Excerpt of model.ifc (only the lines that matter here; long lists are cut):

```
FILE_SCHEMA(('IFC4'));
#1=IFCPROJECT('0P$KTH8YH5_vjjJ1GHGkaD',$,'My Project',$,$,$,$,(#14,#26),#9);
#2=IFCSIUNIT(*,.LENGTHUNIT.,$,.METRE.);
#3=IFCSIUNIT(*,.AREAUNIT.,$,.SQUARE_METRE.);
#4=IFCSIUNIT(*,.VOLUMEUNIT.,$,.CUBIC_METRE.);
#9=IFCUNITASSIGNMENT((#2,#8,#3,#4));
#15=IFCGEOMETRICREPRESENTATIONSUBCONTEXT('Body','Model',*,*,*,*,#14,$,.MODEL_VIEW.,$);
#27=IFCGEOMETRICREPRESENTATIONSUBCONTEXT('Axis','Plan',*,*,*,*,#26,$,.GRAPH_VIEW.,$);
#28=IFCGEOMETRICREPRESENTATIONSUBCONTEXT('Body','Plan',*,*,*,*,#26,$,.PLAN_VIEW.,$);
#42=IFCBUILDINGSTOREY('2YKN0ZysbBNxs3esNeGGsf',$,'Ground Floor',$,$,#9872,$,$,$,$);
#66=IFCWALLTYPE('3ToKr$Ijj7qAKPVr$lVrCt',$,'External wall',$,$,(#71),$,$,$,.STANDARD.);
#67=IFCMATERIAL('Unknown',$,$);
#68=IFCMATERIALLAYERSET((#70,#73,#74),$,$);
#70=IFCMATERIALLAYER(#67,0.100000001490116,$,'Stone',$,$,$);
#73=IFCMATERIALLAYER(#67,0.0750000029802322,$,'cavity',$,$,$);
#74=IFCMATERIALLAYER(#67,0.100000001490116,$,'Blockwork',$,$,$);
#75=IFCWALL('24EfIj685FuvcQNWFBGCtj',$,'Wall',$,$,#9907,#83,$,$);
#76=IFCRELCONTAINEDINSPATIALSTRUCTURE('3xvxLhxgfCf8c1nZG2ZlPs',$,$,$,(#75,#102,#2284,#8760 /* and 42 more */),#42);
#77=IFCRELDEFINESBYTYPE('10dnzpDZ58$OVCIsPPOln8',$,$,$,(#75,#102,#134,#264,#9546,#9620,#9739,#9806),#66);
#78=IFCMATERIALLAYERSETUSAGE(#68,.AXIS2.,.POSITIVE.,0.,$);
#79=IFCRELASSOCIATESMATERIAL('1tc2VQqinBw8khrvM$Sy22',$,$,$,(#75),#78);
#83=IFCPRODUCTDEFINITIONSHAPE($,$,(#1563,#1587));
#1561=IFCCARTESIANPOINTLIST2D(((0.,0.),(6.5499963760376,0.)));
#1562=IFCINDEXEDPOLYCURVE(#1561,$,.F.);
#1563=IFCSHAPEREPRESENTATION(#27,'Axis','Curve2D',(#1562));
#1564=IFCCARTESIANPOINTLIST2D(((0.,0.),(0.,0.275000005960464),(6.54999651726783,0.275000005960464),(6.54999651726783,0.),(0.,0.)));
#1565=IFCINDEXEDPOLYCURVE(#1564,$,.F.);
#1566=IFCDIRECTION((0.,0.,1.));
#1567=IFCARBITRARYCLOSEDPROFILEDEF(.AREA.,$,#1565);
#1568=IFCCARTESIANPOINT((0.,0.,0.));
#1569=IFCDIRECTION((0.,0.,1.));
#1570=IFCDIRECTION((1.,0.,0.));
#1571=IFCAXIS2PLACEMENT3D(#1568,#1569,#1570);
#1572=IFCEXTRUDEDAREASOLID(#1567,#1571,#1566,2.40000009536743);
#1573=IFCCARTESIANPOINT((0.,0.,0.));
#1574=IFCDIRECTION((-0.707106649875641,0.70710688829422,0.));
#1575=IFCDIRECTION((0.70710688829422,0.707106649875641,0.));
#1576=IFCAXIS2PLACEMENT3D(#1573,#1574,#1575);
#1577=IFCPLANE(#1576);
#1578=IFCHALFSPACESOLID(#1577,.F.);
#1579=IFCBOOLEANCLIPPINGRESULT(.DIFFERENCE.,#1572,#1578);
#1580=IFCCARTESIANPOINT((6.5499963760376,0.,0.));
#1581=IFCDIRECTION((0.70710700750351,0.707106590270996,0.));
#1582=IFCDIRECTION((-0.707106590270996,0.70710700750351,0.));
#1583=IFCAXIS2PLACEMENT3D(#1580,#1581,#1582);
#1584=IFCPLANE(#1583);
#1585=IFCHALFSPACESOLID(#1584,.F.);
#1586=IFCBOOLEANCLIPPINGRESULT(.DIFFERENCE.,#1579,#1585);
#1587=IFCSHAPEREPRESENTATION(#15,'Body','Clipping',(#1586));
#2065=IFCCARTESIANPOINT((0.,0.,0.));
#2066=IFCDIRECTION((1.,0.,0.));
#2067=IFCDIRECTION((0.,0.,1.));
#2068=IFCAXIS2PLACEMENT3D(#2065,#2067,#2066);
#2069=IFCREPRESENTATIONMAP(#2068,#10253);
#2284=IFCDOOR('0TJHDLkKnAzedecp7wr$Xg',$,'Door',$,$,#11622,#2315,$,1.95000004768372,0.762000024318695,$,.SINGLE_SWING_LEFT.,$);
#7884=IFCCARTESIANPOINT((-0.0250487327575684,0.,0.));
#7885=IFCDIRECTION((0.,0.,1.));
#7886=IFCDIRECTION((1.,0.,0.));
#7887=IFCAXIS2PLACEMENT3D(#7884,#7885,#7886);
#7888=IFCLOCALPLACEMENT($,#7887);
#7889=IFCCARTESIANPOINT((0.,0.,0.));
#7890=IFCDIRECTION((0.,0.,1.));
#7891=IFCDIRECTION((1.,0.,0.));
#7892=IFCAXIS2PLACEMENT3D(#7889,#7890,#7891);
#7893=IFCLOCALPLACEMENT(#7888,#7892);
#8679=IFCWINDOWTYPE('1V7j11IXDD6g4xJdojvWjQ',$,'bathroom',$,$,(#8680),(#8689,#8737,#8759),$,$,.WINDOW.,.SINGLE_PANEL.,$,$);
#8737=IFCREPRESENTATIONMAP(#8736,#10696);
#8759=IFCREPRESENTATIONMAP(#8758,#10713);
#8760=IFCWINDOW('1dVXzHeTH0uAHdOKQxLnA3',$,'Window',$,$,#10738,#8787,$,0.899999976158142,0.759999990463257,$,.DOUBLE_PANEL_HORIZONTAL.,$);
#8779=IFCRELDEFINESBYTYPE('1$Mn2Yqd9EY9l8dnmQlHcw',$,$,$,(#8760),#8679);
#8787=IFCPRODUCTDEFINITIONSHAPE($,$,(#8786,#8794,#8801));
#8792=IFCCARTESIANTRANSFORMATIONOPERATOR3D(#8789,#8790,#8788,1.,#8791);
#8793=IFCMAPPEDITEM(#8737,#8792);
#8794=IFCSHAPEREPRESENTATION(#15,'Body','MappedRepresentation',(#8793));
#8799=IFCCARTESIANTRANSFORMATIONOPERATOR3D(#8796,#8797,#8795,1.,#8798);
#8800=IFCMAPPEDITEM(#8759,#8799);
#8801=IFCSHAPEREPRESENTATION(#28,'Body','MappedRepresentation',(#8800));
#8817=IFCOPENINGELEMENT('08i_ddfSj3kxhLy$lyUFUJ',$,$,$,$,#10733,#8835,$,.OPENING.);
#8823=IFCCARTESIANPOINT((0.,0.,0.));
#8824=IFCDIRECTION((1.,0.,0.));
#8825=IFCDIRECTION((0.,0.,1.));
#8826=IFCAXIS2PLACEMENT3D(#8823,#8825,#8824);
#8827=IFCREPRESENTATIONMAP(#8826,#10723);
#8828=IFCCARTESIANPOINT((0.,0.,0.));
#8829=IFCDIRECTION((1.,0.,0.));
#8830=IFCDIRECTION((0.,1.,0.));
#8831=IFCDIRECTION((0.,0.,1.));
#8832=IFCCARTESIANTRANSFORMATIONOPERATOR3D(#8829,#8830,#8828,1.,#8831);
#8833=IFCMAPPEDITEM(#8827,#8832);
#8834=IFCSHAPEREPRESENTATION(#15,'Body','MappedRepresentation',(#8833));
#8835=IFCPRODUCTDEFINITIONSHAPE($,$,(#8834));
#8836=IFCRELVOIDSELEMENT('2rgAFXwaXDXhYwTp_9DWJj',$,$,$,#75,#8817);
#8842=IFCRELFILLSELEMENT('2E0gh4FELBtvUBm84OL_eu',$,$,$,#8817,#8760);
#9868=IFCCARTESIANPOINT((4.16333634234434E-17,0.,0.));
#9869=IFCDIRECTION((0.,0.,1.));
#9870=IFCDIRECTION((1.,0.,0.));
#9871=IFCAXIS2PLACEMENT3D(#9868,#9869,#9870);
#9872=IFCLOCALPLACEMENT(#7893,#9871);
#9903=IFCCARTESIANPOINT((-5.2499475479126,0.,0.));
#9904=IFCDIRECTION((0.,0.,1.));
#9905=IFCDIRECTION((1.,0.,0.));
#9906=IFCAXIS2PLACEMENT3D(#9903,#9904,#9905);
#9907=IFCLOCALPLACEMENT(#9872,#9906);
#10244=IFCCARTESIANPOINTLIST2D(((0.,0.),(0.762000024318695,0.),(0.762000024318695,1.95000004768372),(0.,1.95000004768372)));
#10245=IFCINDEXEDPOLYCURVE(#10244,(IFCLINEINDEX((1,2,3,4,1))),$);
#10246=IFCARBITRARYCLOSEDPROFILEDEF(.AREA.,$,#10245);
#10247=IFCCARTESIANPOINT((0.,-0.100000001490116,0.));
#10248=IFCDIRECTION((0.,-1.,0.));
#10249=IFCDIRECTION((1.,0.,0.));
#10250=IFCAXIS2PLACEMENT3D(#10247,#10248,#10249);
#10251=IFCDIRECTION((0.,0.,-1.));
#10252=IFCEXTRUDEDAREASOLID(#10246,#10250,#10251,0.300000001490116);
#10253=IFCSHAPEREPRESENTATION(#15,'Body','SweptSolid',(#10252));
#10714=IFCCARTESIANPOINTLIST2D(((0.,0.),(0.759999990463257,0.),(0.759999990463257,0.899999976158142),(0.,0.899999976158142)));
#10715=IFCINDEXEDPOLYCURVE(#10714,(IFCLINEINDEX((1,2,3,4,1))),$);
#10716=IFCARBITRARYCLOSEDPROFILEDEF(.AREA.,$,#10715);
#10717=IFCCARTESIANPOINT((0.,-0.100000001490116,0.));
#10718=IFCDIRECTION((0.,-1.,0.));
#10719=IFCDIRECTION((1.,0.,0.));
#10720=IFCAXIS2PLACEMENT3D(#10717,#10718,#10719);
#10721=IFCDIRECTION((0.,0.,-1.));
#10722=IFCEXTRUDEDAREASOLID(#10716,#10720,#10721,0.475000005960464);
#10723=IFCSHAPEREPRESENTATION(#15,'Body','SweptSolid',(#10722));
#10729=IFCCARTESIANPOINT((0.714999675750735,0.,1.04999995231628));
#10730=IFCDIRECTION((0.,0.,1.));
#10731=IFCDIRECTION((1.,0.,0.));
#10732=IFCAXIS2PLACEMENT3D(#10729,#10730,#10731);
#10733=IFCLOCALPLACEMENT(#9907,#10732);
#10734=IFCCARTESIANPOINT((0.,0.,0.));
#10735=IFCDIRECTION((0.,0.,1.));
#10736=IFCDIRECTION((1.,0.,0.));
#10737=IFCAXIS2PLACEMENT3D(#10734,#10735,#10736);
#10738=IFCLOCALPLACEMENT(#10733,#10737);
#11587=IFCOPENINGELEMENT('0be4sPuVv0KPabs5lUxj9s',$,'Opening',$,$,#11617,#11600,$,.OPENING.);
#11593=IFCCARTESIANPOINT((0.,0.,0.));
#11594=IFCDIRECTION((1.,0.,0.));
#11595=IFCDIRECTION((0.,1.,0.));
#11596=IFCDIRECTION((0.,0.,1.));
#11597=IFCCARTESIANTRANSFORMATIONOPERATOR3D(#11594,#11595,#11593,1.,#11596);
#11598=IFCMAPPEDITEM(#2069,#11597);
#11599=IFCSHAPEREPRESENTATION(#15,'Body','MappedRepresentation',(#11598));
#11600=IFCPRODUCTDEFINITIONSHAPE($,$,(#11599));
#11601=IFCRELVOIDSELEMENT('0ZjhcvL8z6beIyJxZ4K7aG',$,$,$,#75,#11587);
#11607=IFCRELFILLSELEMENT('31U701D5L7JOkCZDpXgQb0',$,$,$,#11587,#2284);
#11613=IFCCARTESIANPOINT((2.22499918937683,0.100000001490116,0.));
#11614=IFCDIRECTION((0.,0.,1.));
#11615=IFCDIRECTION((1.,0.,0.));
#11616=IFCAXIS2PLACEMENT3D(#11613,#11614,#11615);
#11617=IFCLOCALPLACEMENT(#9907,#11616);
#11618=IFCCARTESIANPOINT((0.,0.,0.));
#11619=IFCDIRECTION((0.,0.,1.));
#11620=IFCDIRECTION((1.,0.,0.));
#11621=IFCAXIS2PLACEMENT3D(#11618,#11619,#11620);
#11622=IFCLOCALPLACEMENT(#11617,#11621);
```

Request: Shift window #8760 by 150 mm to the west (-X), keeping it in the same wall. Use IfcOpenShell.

```python
import ifcopenshell
import ifcopenshell.api.geometry
import ifcopenshell.util.placement

model = ifcopenshell.open("model.ifc")

window = model.by_guid("1dVXzHeTH0uAHdOKQxLnA3")
opening = window.FillsVoids[0].RelatingOpeningElement
wall = opening.VoidsElements[0].RelatingBuildingElement

wall_matrix = ifcopenshell.util.placement.get_local_placement(wall.ObjectPlacement)
shift = wall_matrix[:3, 0] * -0.15
before = ifcopenshell.util.placement.get_local_placement(window.ObjectPlacement)[:3, 3].copy()

# The window is placed relative to its opening, so it follows when the opening moves.
matrix = ifcopenshell.util.placement.get_local_placement(opening.ObjectPlacement)
matrix[:3, 3] += shift
ifcopenshell.api.geometry.edit_object_placement(
    model, product=opening, matrix=matrix, is_si=False, should_transform_children=True
)

after = ifcopenshell.util.placement.get_local_placement(window.ObjectPlacement)[:3, 3]
print("window moved by", (after - before).round(3) + 0.0)

model.write("model-out.ifc")
```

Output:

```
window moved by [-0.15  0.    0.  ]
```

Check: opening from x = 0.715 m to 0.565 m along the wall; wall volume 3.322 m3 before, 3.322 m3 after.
